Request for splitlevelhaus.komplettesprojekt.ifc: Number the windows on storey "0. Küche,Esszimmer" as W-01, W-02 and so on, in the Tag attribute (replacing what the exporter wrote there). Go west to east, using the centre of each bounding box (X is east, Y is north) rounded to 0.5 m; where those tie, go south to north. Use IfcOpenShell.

First a look at what the model holds.

```python
import ifcopenshell
import ifcopenshell.util.element
import ifcopenshell.util.placement

model = ifcopenshell.open("splitlevelhaus.komplettesprojekt.ifc")
print(model.schema)
storey = next(s for s in model.by_type("IfcBuildingStorey") if s.Name == "0. Küche,Esszimmer")
windows = [e for e in ifcopenshell.util.element.get_decomposition(storey) if e.is_a("IfcWindow")]
for e in sorted(windows, key=lambda e: e.id()):
    origin = ifcopenshell.util.placement.get_local_placement(e.ObjectPlacement)[:3, 3]
    print(e.id(), e.Tag, e.Name, origin.round(2) + 0.0, sep=" | ")
```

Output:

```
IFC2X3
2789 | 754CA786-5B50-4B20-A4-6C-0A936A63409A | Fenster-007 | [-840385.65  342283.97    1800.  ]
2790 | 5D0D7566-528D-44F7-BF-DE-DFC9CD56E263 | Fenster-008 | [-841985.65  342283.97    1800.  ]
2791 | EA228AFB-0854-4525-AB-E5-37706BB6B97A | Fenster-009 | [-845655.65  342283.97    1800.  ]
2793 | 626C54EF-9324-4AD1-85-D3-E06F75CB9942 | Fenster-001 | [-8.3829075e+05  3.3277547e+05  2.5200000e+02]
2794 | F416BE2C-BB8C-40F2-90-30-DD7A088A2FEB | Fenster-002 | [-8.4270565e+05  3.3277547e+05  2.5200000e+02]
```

```python
import ifcopenshell
import ifcopenshell.geom
import ifcopenshell.util.element
import ifcopenshell.util.shape

model = ifcopenshell.open("splitlevelhaus.komplettesprojekt.ifc")
settings = ifcopenshell.geom.settings()
settings.set("use-world-coords", True)


def centre(element):
    shape = ifcopenshell.geom.create_shape(settings, element)
    return ifcopenshell.util.shape.get_bbox_centroid(shape.geometry)


storey = next(s for s in model.by_type("IfcBuildingStorey") if s.Name == "0. Küche,Esszimmer")
windows = [e for e in ifcopenshell.util.element.get_decomposition(storey) if e.is_a("IfcWindow")]

# Insertion points can sit at a corner or the storey origin, so sort by the geometry (in metres).
centres = {e: centre(e) for e in windows}
windows.sort(key=lambda e: (round(centres[e][0] / 0.5), centres[e][1]))

for i, e in enumerate(windows, start=1):
    number = f"W-{i:02d}"
    e.Tag = number
    print(e.id(), number)

model.write("splitlevelhaus.komplettesprojekt_v2.ifc")
```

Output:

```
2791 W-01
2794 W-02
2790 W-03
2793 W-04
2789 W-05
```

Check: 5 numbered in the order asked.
